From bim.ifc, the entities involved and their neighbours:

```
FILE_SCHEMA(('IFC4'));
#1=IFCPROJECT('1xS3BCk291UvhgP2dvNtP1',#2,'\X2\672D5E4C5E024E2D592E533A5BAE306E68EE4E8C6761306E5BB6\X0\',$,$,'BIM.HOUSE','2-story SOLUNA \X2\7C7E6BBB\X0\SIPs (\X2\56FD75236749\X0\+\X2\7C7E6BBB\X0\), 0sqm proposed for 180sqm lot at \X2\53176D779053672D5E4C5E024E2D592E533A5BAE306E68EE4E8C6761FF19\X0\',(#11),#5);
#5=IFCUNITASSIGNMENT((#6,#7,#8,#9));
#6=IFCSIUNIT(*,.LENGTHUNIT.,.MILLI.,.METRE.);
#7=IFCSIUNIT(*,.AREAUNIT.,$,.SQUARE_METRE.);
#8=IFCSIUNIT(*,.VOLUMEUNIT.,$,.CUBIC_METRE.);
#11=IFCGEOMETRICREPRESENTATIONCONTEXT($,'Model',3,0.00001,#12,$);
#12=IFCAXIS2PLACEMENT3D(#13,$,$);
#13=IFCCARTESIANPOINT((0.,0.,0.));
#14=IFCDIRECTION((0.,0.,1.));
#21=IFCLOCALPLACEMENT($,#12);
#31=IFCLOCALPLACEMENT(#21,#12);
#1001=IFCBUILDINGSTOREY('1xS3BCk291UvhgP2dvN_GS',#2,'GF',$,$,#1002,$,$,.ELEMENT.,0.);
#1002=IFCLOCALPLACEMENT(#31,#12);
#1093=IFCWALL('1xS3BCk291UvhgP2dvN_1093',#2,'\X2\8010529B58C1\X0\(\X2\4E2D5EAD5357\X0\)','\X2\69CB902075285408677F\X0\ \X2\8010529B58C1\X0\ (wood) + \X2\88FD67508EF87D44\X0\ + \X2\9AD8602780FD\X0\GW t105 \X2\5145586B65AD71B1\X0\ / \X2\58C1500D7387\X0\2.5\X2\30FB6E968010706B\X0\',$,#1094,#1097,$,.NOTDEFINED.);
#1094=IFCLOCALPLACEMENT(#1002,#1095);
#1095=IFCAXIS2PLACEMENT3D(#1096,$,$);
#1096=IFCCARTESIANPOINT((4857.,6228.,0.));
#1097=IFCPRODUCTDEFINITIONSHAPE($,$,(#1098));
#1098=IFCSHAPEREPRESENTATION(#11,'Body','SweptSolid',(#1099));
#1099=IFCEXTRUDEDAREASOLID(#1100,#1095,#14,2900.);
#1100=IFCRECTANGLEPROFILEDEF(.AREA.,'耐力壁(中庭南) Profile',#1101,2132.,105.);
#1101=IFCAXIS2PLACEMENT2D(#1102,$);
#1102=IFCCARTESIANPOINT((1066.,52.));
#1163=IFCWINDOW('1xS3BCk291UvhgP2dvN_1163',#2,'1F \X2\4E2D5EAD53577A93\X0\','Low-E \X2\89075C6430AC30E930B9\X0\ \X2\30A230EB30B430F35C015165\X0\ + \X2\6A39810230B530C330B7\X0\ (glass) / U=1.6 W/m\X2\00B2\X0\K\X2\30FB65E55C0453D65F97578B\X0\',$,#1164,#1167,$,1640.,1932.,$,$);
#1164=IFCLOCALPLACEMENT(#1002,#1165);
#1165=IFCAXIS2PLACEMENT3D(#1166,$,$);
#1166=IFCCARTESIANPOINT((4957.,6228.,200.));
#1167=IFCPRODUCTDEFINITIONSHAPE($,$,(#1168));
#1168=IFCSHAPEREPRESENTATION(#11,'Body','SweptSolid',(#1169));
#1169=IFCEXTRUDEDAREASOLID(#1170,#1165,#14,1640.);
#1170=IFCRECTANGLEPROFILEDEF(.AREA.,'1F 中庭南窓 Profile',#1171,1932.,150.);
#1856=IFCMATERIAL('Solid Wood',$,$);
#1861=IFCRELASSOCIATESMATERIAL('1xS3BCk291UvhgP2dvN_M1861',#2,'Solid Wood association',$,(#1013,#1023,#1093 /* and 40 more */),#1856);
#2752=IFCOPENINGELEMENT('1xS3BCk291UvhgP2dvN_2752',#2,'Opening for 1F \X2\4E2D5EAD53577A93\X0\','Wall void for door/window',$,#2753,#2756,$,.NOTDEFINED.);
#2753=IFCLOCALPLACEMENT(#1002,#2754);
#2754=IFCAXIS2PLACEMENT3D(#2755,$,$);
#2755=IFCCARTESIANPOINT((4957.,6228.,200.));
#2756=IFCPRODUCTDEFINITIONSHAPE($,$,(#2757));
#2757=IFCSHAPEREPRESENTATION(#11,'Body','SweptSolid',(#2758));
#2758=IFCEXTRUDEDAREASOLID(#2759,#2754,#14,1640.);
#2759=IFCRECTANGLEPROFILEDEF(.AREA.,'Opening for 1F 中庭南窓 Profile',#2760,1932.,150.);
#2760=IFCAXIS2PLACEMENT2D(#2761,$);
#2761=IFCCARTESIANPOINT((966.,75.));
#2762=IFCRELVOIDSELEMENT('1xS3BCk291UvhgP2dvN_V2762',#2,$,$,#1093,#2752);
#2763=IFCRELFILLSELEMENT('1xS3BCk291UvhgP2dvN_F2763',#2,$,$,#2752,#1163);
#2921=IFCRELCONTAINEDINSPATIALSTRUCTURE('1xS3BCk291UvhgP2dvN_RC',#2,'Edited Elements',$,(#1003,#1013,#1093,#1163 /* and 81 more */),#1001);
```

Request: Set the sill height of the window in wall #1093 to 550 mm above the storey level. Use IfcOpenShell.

```python
import numpy as np
import ifcopenshell
import ifcopenshell.api.geometry
import ifcopenshell.geom
import ifcopenshell.util.element
import ifcopenshell.util.placement
import ifcopenshell.util.shape
import ifcopenshell.util.unit

model = ifcopenshell.open("bim.ifc")
unit_scale = ifcopenshell.util.unit.calculate_unit_scale(model)

window = model.by_id(1163)
opening = window.FillsVoids[0].RelatingOpeningElement
storey = ifcopenshell.util.element.get_container(window, ifc_class="IfcBuildingStorey")
level = ifcopenshell.util.placement.get_local_placement(storey.ObjectPlacement)[2, 3]

# The opening's origin need not be at the sill, so measure its lowest point.
shape = ifcopenshell.geom.create_shape(ifcopenshell.geom.settings(), opening)
bottom = ifcopenshell.util.shape.get_shape_bottom_elevation(shape, shape.geometry) / unit_scale
dz = level + 550.0 - bottom

shift = np.array([0.0, 0.0, dz])
# The window is not placed relative to its opening, so move both.
for product in (opening, window):
    matrix = ifcopenshell.util.placement.get_local_placement(product.ObjectPlacement)
    matrix[:3, 3] += shift
    ifcopenshell.api.geometry.edit_object_placement(model, product=product, matrix=matrix, is_si=False)

print(f"moved by {dz * unit_scale:+.3f} m")

model.write("bim-out.ifc")
```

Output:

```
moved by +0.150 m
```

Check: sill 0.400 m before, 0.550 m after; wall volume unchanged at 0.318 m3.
